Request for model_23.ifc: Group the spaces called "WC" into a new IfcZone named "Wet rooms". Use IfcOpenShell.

First a look at what the model holds.

```python
import ifcopenshell

model = ifcopenshell.open("model_23.ifc")
print(model.schema)
seen = {}
for space in model.by_type("IfcSpace"):
    seen[space.LongName] = seen.get(space.LongName, 0) + 1
for name, count in sorted(seen.items(), key=str):
    print(count, "x", name)
print("zones:", [z.Name for z in model.by_type("IfcZone")][:20])
```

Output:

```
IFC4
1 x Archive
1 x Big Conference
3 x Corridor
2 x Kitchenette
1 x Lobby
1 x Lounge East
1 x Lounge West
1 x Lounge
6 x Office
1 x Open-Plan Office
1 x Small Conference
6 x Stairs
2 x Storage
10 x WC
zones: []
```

```python
import ifcopenshell
import ifcopenshell.api.group
import ifcopenshell.api.root

model = ifcopenshell.open("model_23.ifc")

names = {"WC"}
spaces = [s for s in model.by_type("IfcSpace") if s.LongName in names]

zone = ifcopenshell.api.root.create_entity(model, ifc_class="IfcZone", name="Wet rooms")
ifcopenshell.api.group.assign_group(model, products=spaces, group=zone)
print(len(spaces), "spaces in", zone.Name)

model.write("model_23_updated.ifc")
```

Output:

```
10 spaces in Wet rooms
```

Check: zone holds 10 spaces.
